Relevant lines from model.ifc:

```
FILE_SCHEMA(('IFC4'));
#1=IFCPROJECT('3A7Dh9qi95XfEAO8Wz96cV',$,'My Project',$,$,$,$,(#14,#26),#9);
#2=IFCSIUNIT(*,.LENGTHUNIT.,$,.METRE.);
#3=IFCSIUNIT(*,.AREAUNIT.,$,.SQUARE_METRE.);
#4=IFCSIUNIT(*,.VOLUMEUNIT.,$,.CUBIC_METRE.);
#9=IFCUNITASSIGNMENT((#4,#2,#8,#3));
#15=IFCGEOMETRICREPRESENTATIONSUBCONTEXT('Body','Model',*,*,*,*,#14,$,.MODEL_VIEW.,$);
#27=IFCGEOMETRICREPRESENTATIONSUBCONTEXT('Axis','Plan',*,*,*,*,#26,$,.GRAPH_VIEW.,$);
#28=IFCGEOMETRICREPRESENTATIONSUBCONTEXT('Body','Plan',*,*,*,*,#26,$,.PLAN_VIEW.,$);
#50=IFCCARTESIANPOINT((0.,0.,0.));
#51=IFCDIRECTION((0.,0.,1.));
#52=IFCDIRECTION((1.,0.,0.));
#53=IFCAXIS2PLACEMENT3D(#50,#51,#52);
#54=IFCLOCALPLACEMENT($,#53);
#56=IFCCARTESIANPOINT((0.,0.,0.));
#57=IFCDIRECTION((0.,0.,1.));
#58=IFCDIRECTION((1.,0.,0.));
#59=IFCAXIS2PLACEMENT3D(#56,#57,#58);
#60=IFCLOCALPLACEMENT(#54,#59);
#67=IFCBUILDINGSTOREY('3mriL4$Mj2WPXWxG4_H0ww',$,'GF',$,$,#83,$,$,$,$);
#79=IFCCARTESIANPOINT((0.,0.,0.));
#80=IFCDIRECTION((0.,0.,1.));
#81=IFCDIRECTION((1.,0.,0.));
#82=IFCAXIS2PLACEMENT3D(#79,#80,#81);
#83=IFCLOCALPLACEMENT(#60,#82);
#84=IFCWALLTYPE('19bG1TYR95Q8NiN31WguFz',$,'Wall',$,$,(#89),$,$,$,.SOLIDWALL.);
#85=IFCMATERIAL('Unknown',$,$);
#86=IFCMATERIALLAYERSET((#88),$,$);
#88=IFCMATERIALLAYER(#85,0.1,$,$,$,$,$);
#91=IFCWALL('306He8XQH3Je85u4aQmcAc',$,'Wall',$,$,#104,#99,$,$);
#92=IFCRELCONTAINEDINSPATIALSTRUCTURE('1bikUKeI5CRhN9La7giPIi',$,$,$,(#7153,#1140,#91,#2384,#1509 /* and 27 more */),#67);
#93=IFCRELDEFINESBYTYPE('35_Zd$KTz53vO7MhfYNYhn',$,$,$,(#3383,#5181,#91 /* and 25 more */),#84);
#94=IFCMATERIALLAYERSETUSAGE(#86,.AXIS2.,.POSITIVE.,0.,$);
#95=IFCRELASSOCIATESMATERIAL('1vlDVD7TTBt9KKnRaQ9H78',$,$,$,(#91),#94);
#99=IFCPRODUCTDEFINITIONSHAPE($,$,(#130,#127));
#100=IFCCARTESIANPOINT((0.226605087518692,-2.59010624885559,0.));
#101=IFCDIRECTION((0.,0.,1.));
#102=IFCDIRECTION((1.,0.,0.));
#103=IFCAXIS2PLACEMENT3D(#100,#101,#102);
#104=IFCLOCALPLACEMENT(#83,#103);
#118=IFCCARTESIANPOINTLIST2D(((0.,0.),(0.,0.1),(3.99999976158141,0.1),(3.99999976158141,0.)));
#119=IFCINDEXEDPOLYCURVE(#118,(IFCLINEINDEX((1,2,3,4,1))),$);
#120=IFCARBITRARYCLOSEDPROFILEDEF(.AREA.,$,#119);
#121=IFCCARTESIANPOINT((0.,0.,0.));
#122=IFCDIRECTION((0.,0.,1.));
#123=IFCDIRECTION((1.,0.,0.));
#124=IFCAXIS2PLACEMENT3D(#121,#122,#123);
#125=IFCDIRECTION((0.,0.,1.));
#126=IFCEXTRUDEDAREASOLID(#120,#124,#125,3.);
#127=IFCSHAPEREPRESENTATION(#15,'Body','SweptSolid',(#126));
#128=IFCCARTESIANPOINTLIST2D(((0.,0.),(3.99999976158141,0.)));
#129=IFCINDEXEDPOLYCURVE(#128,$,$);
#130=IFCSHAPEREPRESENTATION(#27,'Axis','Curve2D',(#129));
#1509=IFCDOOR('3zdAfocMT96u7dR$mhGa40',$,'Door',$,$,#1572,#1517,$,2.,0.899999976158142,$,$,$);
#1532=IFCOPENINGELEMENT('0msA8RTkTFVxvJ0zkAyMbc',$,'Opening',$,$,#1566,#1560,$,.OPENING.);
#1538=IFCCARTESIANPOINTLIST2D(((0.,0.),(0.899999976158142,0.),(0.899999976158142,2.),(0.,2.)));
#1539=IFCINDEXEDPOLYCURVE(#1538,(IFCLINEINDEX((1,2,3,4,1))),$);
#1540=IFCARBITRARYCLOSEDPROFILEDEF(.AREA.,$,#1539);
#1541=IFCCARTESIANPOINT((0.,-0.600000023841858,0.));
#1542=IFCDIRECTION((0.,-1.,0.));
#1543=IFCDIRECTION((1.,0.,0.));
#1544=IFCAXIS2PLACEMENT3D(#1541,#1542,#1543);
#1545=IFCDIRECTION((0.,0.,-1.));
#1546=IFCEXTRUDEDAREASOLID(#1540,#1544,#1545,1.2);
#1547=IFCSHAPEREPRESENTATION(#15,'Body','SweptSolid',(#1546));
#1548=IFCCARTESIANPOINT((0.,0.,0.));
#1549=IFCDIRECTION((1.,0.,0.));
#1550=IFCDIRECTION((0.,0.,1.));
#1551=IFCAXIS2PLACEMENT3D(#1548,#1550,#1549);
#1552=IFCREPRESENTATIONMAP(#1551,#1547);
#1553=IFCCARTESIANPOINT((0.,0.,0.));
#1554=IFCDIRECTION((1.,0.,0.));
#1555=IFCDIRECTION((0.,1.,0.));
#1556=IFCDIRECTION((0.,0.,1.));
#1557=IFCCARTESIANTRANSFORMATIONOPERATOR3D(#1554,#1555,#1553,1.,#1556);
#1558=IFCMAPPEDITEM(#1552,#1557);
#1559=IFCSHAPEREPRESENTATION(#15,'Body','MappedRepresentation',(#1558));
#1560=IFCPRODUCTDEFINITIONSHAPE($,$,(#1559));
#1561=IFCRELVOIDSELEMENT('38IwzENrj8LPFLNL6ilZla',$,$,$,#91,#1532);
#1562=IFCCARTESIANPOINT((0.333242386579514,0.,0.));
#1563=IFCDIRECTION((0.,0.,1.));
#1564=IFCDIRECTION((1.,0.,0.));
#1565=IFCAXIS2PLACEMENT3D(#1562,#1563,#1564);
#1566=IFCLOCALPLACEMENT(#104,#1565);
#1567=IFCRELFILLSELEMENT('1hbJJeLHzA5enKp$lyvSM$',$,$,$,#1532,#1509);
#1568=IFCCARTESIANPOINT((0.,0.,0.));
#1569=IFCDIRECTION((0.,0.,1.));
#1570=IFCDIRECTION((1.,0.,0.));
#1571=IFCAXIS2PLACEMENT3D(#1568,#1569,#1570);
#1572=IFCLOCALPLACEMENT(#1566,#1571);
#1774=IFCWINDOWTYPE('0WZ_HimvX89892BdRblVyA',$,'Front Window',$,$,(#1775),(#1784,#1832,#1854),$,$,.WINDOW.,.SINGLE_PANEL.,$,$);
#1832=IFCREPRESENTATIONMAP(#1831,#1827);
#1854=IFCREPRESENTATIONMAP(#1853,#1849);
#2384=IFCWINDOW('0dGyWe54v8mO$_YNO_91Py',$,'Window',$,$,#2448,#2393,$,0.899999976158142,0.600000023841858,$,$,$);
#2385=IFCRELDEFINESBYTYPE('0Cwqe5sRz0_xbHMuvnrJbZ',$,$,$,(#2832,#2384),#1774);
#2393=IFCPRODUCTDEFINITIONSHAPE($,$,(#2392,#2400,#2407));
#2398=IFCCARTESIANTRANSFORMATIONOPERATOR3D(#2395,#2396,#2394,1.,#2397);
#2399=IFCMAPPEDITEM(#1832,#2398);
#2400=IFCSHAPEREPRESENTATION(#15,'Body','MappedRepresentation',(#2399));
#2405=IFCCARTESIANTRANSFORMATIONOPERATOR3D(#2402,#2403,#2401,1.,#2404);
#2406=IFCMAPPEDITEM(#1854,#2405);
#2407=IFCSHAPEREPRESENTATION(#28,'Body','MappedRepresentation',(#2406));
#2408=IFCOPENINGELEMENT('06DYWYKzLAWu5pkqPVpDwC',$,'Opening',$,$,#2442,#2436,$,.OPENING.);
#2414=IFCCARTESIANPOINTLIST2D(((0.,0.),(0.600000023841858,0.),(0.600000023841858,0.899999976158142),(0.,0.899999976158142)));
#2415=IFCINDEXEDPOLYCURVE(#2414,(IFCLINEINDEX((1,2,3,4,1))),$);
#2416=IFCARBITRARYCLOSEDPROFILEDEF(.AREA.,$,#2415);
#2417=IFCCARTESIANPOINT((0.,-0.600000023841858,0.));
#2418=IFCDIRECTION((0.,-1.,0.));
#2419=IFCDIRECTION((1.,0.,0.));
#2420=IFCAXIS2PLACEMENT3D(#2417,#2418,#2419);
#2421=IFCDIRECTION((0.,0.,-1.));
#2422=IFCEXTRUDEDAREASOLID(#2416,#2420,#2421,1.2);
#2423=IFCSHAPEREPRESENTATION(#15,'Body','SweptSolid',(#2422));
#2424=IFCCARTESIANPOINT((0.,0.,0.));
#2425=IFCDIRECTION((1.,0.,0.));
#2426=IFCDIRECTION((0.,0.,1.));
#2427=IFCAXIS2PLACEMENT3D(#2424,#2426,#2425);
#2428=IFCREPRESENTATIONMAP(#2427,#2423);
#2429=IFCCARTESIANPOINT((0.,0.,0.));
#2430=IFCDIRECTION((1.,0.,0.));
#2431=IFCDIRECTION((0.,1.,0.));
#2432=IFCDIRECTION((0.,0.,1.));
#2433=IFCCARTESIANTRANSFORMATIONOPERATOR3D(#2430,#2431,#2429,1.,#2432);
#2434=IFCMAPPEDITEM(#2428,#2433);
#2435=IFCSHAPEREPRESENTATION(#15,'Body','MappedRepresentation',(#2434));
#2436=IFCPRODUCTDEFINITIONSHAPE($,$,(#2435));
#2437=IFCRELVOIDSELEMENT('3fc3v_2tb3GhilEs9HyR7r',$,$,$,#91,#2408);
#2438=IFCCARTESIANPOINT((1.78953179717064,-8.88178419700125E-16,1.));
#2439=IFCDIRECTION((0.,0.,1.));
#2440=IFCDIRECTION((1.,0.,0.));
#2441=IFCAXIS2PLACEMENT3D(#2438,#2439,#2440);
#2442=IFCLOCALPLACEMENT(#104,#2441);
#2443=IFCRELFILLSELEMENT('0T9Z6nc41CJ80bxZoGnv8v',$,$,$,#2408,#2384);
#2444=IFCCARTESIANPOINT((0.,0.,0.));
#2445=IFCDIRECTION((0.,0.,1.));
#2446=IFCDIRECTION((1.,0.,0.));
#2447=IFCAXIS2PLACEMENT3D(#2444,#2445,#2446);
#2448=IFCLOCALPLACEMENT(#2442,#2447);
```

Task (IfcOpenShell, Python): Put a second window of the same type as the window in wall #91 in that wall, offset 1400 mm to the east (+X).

```python
import ifcopenshell
import ifcopenshell.api.feature
import ifcopenshell.api.geometry
import ifcopenshell.api.root
import ifcopenshell.geom
import ifcopenshell.util.element
import ifcopenshell.util.placement
import ifcopenshell.util.shape
import ifcopenshell.util.unit

model = ifcopenshell.open("model.ifc")
unit_scale = ifcopenshell.util.unit.calculate_unit_scale(model)
settings = ifcopenshell.geom.settings()


def volume(element):
    """Net volume in cubic metres, openings subtracted."""
    shape = ifcopenshell.geom.create_shape(settings, element)
    return ifcopenshell.util.shape.get_volume(shape.geometry)


window = model.by_guid("0dGyWe54v8mO$_YNO_91Py")
opening = window.FillsVoids[0].RelatingOpeningElement
wall = opening.VoidsElements[0].RelatingBuildingElement
before = volume(wall)
shift = ifcopenshell.util.placement.get_local_placement(wall.ObjectPlacement)[:3, 0] * 1.4 / unit_scale

# copy_class copies the void relationship, type, container and properties, but no geometry.
new_opening = ifcopenshell.api.root.copy_class(model, product=opening)
new_opening.Representation = ifcopenshell.util.element.copy_deep(
    model, opening.Representation, exclude=["IfcGeometricRepresentationContext", "IfcRepresentationMap"]
)
new_window = ifcopenshell.api.root.copy_class(model, product=window)
new_window.Representation = ifcopenshell.util.element.copy_deep(
    model, window.Representation, exclude=["IfcGeometricRepresentationContext", "IfcRepresentationMap"]
)
ifcopenshell.api.feature.add_filling(model, opening=new_opening, element=new_window)

for old, new in ((opening, new_opening), (window, new_window)):
    matrix = ifcopenshell.util.placement.get_local_placement(old.ObjectPlacement)
    matrix[:3, 3] += shift
    ifcopenshell.api.geometry.edit_object_placement(model, product=new, matrix=matrix, is_si=False)

after = volume(wall)

print(f"wall volume {before:.3f} -> {after:.3f} m3")

model.write("model_rev.ifc")
```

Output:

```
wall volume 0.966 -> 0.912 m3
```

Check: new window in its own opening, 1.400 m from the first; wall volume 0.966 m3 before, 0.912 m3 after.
